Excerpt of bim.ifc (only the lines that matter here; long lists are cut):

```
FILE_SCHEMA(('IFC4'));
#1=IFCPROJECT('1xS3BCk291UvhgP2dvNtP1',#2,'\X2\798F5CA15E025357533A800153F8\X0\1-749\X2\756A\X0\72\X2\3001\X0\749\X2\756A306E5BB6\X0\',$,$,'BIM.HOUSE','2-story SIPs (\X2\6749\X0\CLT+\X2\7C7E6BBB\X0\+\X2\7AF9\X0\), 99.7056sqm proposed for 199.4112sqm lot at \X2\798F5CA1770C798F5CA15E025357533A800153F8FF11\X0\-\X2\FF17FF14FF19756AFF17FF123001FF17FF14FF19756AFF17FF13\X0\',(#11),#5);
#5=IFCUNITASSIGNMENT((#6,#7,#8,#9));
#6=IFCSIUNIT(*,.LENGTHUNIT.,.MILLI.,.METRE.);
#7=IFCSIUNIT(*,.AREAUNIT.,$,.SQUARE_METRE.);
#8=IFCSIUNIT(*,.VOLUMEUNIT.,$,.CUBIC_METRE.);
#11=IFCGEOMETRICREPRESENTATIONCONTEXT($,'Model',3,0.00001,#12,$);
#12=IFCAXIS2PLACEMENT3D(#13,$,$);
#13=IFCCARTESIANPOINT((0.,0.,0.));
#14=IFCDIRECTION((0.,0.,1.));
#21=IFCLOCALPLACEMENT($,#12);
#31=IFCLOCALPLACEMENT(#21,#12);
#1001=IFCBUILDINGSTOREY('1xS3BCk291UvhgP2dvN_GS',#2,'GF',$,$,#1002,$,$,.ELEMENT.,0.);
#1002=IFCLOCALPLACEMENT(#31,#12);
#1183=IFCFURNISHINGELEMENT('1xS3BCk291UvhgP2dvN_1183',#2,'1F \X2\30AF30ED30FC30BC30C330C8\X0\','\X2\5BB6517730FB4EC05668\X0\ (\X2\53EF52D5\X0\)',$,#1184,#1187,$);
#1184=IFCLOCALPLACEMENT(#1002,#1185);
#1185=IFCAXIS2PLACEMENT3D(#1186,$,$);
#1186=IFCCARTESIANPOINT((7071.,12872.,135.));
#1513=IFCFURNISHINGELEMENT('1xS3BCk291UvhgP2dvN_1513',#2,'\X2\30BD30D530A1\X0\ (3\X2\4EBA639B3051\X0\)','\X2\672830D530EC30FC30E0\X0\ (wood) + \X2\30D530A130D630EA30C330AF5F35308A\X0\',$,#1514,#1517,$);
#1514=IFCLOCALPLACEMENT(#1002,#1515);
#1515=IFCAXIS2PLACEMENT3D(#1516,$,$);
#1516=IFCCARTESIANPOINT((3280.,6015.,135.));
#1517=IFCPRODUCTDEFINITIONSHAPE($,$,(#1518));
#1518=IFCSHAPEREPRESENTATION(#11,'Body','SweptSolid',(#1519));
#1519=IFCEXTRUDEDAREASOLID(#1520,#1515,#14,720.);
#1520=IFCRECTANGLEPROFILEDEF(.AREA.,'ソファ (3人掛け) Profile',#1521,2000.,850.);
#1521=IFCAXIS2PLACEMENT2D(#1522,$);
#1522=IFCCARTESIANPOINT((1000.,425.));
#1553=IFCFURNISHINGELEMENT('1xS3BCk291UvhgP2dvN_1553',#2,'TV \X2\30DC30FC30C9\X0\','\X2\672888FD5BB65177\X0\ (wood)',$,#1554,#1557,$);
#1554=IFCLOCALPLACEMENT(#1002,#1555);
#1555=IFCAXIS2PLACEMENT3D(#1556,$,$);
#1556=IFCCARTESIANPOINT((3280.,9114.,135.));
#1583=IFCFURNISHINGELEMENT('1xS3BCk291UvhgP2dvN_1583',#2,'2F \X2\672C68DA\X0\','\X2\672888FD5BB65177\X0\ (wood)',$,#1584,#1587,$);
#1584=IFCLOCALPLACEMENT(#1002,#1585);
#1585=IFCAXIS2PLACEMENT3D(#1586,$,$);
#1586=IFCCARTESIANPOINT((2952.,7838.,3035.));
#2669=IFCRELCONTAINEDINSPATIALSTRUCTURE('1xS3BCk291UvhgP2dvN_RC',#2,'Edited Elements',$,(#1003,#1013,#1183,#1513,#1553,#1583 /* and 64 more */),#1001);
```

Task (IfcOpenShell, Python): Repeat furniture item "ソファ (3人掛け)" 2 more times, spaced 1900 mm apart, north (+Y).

```python
import numpy as np
import ifcopenshell
import ifcopenshell.api.geometry
import ifcopenshell.api.root
import ifcopenshell.util.element
import ifcopenshell.util.placement

model = ifcopenshell.open("bim.ifc")


def reuse_history(source, copy):
    """copy_class also copies each property set's owner history, people and application; keep the originals."""
    for rel in copy.IsDefinedBy:
        if rel.is_a("IfcRelDefinesByProperties") and (history := rel.RelatingPropertyDefinition.OwnerHistory):
            rel.RelatingPropertyDefinition.OwnerHistory = source.OwnerHistory
            ifcopenshell.util.element.remove_deep2(model, history)


source = model.by_guid("1xS3BCk291UvhgP2dvN_1513")
base = ifcopenshell.util.placement.get_local_placement(source.ObjectPlacement)
step = np.array([0.0, 1.0, 0.0]) * 1900.0

for i in range(1, 3):
    copy = ifcopenshell.api.root.copy_class(model, product=source)
    copy.Representation = ifcopenshell.util.element.copy_deep(
        model, source.Representation, exclude=["IfcGeometricRepresentationContext", "IfcRepresentationMap"]
    )
    reuse_history(source, copy)
    matrix = base.copy()
    matrix[:3, 3] += i * step
    print("added at", matrix[:3, 3].round(3) + 0.0)
    ifcopenshell.api.geometry.edit_object_placement(model, product=copy, matrix=matrix, is_si=False)

model.write("bim_v2.ifc")
```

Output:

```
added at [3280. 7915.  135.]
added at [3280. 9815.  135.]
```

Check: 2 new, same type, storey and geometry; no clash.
